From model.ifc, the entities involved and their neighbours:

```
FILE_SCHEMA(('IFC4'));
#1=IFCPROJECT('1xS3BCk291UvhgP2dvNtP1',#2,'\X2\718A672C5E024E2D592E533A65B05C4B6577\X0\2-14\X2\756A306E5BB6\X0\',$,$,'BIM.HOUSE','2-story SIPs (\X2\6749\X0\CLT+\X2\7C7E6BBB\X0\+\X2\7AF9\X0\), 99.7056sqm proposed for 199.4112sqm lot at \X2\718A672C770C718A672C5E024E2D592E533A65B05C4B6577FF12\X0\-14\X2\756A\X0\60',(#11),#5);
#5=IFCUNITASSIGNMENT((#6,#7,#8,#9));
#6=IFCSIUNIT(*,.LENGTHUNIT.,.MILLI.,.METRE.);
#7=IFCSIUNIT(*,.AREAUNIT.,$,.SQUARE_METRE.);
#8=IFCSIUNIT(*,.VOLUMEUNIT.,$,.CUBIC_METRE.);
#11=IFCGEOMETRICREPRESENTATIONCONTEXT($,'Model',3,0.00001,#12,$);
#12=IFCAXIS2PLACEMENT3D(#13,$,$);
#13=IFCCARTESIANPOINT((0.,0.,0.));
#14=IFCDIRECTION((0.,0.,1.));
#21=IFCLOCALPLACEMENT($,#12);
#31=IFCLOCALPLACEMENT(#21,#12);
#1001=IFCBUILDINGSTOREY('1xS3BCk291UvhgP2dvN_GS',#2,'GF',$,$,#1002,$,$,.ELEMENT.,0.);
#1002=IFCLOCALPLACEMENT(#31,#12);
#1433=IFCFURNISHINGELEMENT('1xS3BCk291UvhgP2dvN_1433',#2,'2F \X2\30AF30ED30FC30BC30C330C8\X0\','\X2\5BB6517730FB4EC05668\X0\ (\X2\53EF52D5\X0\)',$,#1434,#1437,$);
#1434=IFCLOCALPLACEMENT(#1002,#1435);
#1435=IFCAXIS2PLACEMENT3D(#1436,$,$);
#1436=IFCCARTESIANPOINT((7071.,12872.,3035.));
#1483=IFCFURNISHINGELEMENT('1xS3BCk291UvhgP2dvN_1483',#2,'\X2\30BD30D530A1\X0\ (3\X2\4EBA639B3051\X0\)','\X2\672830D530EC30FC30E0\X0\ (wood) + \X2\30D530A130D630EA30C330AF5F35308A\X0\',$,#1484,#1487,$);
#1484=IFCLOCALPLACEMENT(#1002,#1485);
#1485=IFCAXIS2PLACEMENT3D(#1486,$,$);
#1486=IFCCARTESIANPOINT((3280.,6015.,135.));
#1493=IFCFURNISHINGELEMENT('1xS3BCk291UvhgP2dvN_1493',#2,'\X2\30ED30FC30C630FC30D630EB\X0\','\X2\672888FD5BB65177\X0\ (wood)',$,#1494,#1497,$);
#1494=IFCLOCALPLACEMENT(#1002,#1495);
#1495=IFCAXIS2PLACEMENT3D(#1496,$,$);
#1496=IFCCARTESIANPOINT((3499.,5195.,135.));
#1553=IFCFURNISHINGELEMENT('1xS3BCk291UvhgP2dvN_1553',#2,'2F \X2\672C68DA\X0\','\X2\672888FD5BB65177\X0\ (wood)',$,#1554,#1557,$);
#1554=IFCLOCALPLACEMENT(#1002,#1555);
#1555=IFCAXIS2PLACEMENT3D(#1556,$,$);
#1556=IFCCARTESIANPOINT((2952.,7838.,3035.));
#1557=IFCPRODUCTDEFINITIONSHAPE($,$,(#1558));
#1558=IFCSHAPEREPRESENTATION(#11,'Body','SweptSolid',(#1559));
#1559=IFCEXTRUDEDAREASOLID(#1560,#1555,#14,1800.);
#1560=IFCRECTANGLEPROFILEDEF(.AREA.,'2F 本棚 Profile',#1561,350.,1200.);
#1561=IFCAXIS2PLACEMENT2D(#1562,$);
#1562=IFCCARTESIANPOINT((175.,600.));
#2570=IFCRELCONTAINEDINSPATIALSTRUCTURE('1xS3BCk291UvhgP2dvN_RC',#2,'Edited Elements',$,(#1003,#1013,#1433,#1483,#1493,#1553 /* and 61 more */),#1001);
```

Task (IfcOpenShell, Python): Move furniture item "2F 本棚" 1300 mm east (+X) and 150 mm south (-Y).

```python
import ifcopenshell
import ifcopenshell.api.geometry
import ifcopenshell.util.placement
import ifcopenshell.util.unit

model = ifcopenshell.open("model.ifc")
unit_scale = ifcopenshell.util.unit.calculate_unit_scale(model)

item = model.by_guid("1xS3BCk291UvhgP2dvN_1553")
matrix = ifcopenshell.util.placement.get_local_placement(item.ObjectPlacement)
matrix[0, 3] += 1.3 / unit_scale
matrix[1, 3] -= 0.15 / unit_scale
ifcopenshell.api.geometry.edit_object_placement(model, product=item, matrix=matrix, is_si=False)

print(ifcopenshell.util.placement.get_local_placement(item.ObjectPlacement).round(3) + 0.0)

model.write("model_updated.ifc")
```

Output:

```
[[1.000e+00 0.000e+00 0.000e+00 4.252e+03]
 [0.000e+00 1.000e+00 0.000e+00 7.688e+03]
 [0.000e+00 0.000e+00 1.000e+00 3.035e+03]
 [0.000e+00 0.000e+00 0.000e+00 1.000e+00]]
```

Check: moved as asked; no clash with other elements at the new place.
